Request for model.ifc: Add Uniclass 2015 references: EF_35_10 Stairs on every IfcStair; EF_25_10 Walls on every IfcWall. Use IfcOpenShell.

First a look at what the model holds.

```python
import ifcopenshell

model = ifcopenshell.open("model.ifc")
print(model.schema)
print("classifications:", [c.Name for c in model.by_type("IfcClassification")])
for ifc_class in ("IfcDoor", "IfcRoof", "IfcStair", "IfcWall", "IfcWindow"):
    print(ifc_class, len(model.by_type(ifc_class)))
```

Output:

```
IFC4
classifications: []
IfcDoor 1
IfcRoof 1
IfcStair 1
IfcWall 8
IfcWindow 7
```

```python
import ifcopenshell
import ifcopenshell.api.classification

model = ifcopenshell.open("model.ifc")

system = ifcopenshell.api.classification.add_classification(model, classification="Uniclass 2015")

codes = {
    "IfcStair": ("EF_35_10", "Stairs"),
    "IfcWall": ("EF_25_10", "Walls"),
}
for ifc_class, (code, name) in codes.items():
    products = model.by_type(ifc_class)
    ifcopenshell.api.classification.add_reference(
        model, products=products, classification=system, identification=code, name=name
    )
    print(code, len(products))

model.write("model_v2.ifc")
```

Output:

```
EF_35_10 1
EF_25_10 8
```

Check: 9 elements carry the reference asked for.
